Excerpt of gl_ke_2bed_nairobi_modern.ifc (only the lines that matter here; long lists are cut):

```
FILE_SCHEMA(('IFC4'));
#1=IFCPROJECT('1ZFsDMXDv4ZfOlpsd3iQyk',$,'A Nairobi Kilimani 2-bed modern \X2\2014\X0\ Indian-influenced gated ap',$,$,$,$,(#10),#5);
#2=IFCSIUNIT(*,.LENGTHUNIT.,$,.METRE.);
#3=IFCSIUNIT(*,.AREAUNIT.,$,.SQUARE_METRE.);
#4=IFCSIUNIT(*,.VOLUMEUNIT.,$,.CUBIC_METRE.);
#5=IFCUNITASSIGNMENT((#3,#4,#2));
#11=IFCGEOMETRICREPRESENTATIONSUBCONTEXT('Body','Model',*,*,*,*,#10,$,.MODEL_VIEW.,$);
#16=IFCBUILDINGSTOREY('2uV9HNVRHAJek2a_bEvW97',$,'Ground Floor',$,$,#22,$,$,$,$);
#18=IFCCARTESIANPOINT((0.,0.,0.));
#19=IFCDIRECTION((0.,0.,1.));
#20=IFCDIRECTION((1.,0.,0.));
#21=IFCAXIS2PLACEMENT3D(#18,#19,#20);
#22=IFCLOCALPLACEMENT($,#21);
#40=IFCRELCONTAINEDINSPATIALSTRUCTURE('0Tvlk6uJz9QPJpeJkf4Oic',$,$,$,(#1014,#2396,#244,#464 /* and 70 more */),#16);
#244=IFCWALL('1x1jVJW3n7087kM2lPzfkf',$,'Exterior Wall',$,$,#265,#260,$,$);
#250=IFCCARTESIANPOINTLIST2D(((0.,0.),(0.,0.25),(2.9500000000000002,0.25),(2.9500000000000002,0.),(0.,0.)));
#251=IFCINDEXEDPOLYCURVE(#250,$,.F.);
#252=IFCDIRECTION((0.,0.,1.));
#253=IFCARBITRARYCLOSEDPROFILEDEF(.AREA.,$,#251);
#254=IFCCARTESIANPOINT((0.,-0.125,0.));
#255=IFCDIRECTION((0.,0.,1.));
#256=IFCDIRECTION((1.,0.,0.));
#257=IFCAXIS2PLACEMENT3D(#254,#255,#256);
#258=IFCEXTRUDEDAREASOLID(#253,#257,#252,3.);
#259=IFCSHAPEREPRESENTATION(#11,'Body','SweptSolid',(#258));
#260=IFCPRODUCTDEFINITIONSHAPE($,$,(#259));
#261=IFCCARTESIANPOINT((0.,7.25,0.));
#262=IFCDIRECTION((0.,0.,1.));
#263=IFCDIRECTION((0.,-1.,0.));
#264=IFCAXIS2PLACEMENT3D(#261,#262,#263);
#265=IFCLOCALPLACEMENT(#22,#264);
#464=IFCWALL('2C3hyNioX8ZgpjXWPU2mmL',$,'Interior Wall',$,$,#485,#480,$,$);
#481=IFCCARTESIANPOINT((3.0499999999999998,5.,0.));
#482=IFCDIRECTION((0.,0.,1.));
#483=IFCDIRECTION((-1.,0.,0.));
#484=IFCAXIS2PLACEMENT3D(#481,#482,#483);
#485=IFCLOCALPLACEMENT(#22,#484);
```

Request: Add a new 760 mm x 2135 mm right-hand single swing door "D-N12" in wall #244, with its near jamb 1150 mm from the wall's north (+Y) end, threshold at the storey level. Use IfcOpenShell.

```python
import numpy as np
import ifcopenshell
import ifcopenshell.api.feature
import ifcopenshell.api.geometry
import ifcopenshell.api.root
import ifcopenshell.api.spatial
import ifcopenshell.geom
import ifcopenshell.util.element
import ifcopenshell.util.placement
import ifcopenshell.util.representation
import ifcopenshell.util.shape
import ifcopenshell.util.unit

model = ifcopenshell.open("gl_ke_2bed_nairobi_modern.ifc")
unit_scale = ifcopenshell.util.unit.calculate_unit_scale(model)
settings = ifcopenshell.geom.settings()


def volume(element):
    """Net volume in cubic metres, openings subtracted."""
    shape = ifcopenshell.geom.create_shape(settings, element)
    return ifcopenshell.util.shape.get_volume(shape.geometry)


wall = model.by_guid("1x1jVJW3n7087kM2lPzfkf")
storey = ifcopenshell.util.element.get_container(wall, ifc_class="IfcBuildingStorey")
context = ifcopenshell.util.representation.get_context(model, "Model", "Body", "MODEL_VIEW")
before = volume(wall)

width, height, from_end, sill = 0.76, 2.135, 1.15, 0.0  # metres

# The wall runs along its own X axis, and the end named is its -X end.
wall_shape = ifcopenshell.geom.create_shape(settings, wall)
x, y, z = ifcopenshell.util.shape.get_vertices(wall_shape.geometry).T
start = x.min() + from_end
face, thickness = float(y.min()), float(y.max() - y.min())
wall_matrix = ifcopenshell.util.placement.get_local_placement(wall.ObjectPlacement)
level = ifcopenshell.util.placement.get_local_placement(storey.ObjectPlacement)[2, 3]


def in_wall(x, y):
    """Placement at x, y metres in the wall's axes, at sill height."""
    matrix = wall_matrix.copy()
    matrix[:, 3] = wall_matrix @ np.array([x / unit_scale, y / unit_scale, 0.0, 1.0])
    matrix[2, 3] = level + sill / unit_scale
    return matrix


# Opening: a box that overshoots both wall faces by 50 mm.
opening = ifcopenshell.api.root.create_entity(model, ifc_class="IfcOpeningElement", predefined_type="OPENING")
box = ifcopenshell.api.geometry.add_wall_representation(
    model, context=context, length=width, height=height, thickness=thickness + 0.1
)
ifcopenshell.api.geometry.assign_representation(model, product=opening, representation=box)
ifcopenshell.api.geometry.edit_object_placement(model, product=opening, matrix=in_wall(start, face - 0.05), is_si=False)
ifcopenshell.api.feature.add_feature(model, feature=opening, element=wall)

door = ifcopenshell.api.root.create_entity(model, ifc_class="IfcDoor", name="D-N12", predefined_type="DOOR")
door.OverallWidth, door.OverallHeight = width / unit_scale, height / unit_scale
door.OperationType = "SINGLE_SWING_RIGHT"
body = ifcopenshell.api.geometry.add_door_representation(
    model,
    context=context,
    overall_width=door.OverallWidth,
    overall_height=door.OverallHeight,
    operation_type="SINGLE_SWING_RIGHT",
    lining_properties={"LiningDepth": thickness / unit_scale, "ThresholdDepth": thickness / unit_scale},
)
ifcopenshell.api.geometry.assign_representation(model, product=door, representation=body)
ifcopenshell.api.spatial.assign_container(model, products=[door], relating_structure=storey)
ifcopenshell.api.feature.add_filling(model, opening=opening, element=door)

# The lining spans the wall, so the door starts at the wall face.
ifcopenshell.api.geometry.edit_object_placement(model, product=door, matrix=in_wall(start, face), is_si=False)

after = volume(wall)

print(f"wall volume {before:.3f} -> {after:.3f} m3")

model.write("gl_ke_2bed_nairobi_modern-out.ifc")
```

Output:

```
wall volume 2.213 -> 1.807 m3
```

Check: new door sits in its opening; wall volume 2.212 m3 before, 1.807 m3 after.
